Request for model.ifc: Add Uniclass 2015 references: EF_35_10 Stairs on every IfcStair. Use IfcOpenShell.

First a look at what the model holds.

```python
import ifcopenshell

model = ifcopenshell.open("model.ifc")
print(model.schema)
print("classifications:", [c.Name for c in model.by_type("IfcClassification")])
for ifc_class in ("IfcDoor", "IfcRoof", "IfcStair", "IfcWall", "IfcWindow"):
    print(ifc_class, len(model.by_type(ifc_class)))
```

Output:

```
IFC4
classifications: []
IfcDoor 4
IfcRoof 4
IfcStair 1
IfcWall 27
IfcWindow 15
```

```python
import ifcopenshell
import ifcopenshell.api.classification

model = ifcopenshell.open("model.ifc")

system = ifcopenshell.api.classification.add_classification(model, classification="Uniclass 2015")

codes = {
    "IfcStair": ("EF_35_10", "Stairs"),
}
for ifc_class, (code, name) in codes.items():
    products = model.by_type(ifc_class)
    ifcopenshell.api.classification.add_reference(
        model, products=products, classification=system, identification=code, name=name
    )
    print(code, len(products))

model.write("model_edited.ifc")
```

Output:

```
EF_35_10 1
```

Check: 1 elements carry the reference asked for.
